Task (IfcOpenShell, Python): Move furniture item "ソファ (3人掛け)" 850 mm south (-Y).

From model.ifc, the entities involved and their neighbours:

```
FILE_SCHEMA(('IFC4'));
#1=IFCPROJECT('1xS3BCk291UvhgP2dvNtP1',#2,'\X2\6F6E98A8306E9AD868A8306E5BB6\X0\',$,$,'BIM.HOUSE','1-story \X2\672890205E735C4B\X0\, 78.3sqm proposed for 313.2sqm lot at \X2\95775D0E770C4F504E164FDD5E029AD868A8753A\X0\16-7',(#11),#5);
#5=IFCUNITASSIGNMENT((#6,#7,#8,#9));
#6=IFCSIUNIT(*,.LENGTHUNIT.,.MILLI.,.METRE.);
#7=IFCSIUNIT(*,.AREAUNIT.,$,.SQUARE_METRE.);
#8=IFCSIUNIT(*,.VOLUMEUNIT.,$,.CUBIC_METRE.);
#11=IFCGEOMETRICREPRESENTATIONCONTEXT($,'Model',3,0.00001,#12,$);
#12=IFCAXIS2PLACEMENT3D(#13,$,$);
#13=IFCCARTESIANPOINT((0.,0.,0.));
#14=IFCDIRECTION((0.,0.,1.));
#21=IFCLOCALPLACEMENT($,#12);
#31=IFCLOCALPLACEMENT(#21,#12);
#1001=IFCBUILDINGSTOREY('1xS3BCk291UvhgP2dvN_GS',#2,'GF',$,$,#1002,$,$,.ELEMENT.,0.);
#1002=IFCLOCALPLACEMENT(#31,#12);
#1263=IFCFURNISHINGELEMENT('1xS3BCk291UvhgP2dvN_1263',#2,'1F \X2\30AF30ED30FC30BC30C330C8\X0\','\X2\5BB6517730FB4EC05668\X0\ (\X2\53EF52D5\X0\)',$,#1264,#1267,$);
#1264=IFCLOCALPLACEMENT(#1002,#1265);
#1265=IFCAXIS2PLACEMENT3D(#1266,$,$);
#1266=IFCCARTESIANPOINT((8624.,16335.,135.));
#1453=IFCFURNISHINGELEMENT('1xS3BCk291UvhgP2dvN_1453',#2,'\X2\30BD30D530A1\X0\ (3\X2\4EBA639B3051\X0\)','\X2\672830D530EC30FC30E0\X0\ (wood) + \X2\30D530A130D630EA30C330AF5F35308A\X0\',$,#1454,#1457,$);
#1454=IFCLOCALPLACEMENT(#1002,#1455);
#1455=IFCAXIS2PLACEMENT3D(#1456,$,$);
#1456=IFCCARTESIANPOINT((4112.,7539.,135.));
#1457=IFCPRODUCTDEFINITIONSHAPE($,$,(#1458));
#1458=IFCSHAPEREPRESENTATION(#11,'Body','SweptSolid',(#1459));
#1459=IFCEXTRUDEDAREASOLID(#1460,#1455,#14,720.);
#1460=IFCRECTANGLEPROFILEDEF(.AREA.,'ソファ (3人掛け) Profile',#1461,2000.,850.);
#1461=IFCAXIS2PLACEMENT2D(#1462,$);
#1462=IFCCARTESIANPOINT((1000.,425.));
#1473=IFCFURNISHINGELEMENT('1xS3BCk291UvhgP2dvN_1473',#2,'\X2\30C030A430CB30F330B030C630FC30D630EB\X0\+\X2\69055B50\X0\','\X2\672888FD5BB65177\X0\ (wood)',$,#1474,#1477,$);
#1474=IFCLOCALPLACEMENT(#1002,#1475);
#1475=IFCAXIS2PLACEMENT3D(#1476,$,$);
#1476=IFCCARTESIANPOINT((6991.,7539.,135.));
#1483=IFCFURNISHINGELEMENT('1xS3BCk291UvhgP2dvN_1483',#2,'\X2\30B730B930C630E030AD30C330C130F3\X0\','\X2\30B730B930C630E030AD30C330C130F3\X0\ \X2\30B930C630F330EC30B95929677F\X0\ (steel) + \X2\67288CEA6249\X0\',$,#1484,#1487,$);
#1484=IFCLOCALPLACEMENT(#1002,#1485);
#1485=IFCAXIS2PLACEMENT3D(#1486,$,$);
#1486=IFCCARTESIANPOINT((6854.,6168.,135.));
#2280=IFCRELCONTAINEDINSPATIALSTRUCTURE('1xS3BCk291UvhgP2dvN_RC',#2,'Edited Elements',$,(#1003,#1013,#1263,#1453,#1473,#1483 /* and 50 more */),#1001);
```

```python
import ifcopenshell
import ifcopenshell.api.geometry
import ifcopenshell.util.placement

model = ifcopenshell.open("model.ifc")

item = model.by_guid("1xS3BCk291UvhgP2dvN_1453")
matrix = ifcopenshell.util.placement.get_local_placement(item.ObjectPlacement)
matrix[1, 3] -= 850.0
ifcopenshell.api.geometry.edit_object_placement(model, product=item, matrix=matrix, is_si=False)

print(ifcopenshell.util.placement.get_local_placement(item.ObjectPlacement).round(3) + 0.0)

model.write("model_edited.ifc")
```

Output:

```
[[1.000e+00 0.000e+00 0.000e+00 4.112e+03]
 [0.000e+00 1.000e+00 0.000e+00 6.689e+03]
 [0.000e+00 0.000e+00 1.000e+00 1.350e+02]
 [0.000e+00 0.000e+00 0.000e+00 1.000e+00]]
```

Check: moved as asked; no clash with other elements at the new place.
